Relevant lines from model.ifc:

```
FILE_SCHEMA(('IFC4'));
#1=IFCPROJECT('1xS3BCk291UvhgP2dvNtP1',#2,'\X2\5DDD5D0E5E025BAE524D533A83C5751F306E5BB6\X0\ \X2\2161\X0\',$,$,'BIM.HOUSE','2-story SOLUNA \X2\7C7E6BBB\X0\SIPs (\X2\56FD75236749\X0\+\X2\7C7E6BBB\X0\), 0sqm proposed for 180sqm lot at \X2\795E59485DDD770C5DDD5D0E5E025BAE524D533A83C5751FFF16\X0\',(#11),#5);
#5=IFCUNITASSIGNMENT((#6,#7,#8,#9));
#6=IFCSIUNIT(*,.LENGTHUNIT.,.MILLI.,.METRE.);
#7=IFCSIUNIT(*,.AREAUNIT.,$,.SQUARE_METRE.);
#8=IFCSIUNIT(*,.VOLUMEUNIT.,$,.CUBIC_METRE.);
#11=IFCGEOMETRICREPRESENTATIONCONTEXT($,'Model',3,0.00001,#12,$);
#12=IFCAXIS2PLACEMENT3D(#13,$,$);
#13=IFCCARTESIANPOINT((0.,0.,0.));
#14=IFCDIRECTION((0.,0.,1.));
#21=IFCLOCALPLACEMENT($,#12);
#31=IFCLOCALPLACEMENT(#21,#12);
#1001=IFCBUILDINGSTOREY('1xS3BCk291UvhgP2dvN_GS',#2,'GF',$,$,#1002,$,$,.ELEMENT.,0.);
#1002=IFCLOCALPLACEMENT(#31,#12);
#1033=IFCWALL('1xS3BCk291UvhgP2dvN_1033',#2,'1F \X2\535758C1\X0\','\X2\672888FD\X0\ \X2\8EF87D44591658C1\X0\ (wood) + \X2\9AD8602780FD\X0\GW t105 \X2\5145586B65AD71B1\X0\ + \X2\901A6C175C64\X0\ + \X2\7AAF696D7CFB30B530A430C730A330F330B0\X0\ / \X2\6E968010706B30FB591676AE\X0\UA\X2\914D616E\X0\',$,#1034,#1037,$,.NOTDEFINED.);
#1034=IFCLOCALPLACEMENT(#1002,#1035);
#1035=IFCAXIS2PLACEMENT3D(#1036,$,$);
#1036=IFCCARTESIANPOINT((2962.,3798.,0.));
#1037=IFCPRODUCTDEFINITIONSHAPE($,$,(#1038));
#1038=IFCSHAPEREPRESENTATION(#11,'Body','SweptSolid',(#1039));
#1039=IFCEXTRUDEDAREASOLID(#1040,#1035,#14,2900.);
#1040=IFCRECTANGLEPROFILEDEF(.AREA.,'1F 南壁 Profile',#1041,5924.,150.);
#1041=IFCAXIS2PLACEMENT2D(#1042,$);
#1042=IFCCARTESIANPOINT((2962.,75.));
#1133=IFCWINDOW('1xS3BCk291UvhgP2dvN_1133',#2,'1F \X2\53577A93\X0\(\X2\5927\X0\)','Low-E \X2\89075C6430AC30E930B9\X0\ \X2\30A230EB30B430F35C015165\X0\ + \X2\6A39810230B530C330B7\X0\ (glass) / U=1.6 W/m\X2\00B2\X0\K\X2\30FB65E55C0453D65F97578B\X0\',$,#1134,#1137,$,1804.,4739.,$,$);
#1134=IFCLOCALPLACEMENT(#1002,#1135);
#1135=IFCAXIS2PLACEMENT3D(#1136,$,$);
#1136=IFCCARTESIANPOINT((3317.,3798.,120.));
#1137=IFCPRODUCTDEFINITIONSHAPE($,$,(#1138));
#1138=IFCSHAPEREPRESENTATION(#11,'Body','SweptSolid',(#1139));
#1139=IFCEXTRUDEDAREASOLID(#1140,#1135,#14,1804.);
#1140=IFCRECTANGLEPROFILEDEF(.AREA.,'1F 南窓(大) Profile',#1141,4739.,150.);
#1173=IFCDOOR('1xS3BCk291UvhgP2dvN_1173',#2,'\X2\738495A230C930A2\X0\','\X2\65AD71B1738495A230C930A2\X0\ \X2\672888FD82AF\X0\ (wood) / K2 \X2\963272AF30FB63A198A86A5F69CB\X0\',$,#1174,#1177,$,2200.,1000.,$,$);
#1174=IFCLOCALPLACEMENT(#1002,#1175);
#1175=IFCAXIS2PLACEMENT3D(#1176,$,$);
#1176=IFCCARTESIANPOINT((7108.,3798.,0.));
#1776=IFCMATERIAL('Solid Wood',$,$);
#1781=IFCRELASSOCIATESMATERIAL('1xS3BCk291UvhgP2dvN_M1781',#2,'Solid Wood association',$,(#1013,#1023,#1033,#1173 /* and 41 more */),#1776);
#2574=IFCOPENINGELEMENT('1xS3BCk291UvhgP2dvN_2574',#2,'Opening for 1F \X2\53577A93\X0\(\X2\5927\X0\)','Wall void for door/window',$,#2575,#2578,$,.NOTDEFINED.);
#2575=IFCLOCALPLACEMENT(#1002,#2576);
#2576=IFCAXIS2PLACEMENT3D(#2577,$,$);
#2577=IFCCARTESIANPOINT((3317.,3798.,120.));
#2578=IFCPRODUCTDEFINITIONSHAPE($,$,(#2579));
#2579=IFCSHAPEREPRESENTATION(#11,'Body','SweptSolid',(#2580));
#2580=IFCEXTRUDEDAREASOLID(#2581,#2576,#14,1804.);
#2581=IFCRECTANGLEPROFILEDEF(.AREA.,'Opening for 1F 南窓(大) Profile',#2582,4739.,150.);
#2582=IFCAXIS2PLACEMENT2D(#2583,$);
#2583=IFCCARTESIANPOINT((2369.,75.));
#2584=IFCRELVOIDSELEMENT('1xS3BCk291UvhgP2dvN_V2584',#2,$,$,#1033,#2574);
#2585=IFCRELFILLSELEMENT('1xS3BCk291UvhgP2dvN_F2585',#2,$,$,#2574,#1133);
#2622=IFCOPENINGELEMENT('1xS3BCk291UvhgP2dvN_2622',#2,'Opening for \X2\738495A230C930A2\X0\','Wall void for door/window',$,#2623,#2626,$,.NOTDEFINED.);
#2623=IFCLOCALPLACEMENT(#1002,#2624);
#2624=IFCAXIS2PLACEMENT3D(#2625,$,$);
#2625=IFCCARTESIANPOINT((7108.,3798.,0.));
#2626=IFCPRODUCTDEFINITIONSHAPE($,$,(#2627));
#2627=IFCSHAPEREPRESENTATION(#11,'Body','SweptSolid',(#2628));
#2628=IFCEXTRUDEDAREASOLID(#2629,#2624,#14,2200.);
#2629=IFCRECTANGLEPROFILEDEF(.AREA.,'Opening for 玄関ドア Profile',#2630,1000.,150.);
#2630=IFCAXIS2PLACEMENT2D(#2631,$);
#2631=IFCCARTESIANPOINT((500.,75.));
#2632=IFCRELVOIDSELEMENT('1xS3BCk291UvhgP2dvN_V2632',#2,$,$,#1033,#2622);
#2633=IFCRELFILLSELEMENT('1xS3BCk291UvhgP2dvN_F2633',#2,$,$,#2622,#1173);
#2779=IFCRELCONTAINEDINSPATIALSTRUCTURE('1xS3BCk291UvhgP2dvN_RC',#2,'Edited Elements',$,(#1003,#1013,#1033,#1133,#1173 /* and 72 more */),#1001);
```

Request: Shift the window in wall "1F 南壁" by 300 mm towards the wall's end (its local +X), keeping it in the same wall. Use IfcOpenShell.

```python
import ifcopenshell
import ifcopenshell.api.geometry
import ifcopenshell.util.placement

model = ifcopenshell.open("model.ifc")

window = model.by_guid("1xS3BCk291UvhgP2dvN_1133")
opening = window.FillsVoids[0].RelatingOpeningElement
wall = opening.VoidsElements[0].RelatingBuildingElement

wall_matrix = ifcopenshell.util.placement.get_local_placement(wall.ObjectPlacement)
shift = wall_matrix[:3, 0] * 300.0
before = ifcopenshell.util.placement.get_local_placement(window.ObjectPlacement)[:3, 3].copy()

# The window is not placed relative to its opening, so move both.
for product in (opening, window):
    matrix = ifcopenshell.util.placement.get_local_placement(product.ObjectPlacement)
    matrix[:3, 3] += shift
    ifcopenshell.api.geometry.edit_object_placement(model, product=product, matrix=matrix, is_si=False)

after = ifcopenshell.util.placement.get_local_placement(window.ObjectPlacement)[:3, 3]
print("window moved by", (after - before).round(3) + 0.0)

model.write("model_rev.ifc")
```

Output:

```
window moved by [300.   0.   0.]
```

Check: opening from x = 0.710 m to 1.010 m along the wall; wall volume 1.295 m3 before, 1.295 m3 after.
